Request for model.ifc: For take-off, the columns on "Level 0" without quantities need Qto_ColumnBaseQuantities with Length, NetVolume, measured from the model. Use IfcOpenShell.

First a look at what the model holds.

```python
import ifcopenshell
import ifcopenshell.util.element
import ifcopenshell.util.unit

model = ifcopenshell.open("model.ifc")
print(model.schema)
for unit_type in ("LENGTHUNIT", "AREAUNIT", "VOLUMEUNIT"):
    print(unit_type, ifcopenshell.util.unit.calculate_unit_scale(model, unit_type))
storey = next(s for s in model.by_type("IfcBuildingStorey") if s.Name == "Level 0")
columns = [e for e in ifcopenshell.util.element.get_decomposition(storey) if e.is_a("IfcColumn")]
for e in sorted(columns, key=lambda e: e.id()):
    print(e.id(), e.is_a(), e.Name, list(ifcopenshell.util.element.get_psets(e, qtos_only=True)), sep=" | ")
```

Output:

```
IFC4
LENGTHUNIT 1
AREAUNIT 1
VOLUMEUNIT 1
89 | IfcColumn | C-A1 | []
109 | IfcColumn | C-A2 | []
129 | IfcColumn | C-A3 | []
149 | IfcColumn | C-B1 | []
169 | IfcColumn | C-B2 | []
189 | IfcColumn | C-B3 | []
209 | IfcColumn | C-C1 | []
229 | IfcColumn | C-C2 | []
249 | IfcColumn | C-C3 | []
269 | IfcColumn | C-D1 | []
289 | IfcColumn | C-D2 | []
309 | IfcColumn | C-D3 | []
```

```python
import ifcopenshell
import ifcopenshell.api.pset
import ifcopenshell.geom
import ifcopenshell.util.element
import ifcopenshell.util.shape
import ifcopenshell.util.unit

model = ifcopenshell.open("model.ifc")
unit_scale = ifcopenshell.util.unit.calculate_unit_scale(model)
volume_scale = ifcopenshell.util.unit.calculate_unit_scale(model, "VOLUMEUNIT")
settings = ifcopenshell.geom.settings()

storey = next(s for s in model.by_type("IfcBuildingStorey") if s.Name == "Level 0")
columns = [e for e in ifcopenshell.util.element.get_decomposition(storey) if e.is_a("IfcColumn")]

for e in sorted(columns, key=lambda e: e.id()):
    if ifcopenshell.util.element.get_psets(e, qtos_only=True, should_inherit=False):
        continue
    # Geometry comes back in metres, in the element's own axes.
    shape = ifcopenshell.geom.create_shape(settings, e)
    values = {
        "Length": ifcopenshell.util.shape.get_z(shape.geometry) / unit_scale,
        "NetVolume": ifcopenshell.util.shape.get_volume(shape.geometry) / volume_scale,
    }
    qto = ifcopenshell.api.pset.add_qto(model, product=e, name="Qto_ColumnBaseQuantities")
    ifcopenshell.api.pset.edit_qto(model, qto=qto, properties=values)
    print(e.id(), {k: round(v, 3) for k, v in values.items()})

model.write("model_v2.ifc")
```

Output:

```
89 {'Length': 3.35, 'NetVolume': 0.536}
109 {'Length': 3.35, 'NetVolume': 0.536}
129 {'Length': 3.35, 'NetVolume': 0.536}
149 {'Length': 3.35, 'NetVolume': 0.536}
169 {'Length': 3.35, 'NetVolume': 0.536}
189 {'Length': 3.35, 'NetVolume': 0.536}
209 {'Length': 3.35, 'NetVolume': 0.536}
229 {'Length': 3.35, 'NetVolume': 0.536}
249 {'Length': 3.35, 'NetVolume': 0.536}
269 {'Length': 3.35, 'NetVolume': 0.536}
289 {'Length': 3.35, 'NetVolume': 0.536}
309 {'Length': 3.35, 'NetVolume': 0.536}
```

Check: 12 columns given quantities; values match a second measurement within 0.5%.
